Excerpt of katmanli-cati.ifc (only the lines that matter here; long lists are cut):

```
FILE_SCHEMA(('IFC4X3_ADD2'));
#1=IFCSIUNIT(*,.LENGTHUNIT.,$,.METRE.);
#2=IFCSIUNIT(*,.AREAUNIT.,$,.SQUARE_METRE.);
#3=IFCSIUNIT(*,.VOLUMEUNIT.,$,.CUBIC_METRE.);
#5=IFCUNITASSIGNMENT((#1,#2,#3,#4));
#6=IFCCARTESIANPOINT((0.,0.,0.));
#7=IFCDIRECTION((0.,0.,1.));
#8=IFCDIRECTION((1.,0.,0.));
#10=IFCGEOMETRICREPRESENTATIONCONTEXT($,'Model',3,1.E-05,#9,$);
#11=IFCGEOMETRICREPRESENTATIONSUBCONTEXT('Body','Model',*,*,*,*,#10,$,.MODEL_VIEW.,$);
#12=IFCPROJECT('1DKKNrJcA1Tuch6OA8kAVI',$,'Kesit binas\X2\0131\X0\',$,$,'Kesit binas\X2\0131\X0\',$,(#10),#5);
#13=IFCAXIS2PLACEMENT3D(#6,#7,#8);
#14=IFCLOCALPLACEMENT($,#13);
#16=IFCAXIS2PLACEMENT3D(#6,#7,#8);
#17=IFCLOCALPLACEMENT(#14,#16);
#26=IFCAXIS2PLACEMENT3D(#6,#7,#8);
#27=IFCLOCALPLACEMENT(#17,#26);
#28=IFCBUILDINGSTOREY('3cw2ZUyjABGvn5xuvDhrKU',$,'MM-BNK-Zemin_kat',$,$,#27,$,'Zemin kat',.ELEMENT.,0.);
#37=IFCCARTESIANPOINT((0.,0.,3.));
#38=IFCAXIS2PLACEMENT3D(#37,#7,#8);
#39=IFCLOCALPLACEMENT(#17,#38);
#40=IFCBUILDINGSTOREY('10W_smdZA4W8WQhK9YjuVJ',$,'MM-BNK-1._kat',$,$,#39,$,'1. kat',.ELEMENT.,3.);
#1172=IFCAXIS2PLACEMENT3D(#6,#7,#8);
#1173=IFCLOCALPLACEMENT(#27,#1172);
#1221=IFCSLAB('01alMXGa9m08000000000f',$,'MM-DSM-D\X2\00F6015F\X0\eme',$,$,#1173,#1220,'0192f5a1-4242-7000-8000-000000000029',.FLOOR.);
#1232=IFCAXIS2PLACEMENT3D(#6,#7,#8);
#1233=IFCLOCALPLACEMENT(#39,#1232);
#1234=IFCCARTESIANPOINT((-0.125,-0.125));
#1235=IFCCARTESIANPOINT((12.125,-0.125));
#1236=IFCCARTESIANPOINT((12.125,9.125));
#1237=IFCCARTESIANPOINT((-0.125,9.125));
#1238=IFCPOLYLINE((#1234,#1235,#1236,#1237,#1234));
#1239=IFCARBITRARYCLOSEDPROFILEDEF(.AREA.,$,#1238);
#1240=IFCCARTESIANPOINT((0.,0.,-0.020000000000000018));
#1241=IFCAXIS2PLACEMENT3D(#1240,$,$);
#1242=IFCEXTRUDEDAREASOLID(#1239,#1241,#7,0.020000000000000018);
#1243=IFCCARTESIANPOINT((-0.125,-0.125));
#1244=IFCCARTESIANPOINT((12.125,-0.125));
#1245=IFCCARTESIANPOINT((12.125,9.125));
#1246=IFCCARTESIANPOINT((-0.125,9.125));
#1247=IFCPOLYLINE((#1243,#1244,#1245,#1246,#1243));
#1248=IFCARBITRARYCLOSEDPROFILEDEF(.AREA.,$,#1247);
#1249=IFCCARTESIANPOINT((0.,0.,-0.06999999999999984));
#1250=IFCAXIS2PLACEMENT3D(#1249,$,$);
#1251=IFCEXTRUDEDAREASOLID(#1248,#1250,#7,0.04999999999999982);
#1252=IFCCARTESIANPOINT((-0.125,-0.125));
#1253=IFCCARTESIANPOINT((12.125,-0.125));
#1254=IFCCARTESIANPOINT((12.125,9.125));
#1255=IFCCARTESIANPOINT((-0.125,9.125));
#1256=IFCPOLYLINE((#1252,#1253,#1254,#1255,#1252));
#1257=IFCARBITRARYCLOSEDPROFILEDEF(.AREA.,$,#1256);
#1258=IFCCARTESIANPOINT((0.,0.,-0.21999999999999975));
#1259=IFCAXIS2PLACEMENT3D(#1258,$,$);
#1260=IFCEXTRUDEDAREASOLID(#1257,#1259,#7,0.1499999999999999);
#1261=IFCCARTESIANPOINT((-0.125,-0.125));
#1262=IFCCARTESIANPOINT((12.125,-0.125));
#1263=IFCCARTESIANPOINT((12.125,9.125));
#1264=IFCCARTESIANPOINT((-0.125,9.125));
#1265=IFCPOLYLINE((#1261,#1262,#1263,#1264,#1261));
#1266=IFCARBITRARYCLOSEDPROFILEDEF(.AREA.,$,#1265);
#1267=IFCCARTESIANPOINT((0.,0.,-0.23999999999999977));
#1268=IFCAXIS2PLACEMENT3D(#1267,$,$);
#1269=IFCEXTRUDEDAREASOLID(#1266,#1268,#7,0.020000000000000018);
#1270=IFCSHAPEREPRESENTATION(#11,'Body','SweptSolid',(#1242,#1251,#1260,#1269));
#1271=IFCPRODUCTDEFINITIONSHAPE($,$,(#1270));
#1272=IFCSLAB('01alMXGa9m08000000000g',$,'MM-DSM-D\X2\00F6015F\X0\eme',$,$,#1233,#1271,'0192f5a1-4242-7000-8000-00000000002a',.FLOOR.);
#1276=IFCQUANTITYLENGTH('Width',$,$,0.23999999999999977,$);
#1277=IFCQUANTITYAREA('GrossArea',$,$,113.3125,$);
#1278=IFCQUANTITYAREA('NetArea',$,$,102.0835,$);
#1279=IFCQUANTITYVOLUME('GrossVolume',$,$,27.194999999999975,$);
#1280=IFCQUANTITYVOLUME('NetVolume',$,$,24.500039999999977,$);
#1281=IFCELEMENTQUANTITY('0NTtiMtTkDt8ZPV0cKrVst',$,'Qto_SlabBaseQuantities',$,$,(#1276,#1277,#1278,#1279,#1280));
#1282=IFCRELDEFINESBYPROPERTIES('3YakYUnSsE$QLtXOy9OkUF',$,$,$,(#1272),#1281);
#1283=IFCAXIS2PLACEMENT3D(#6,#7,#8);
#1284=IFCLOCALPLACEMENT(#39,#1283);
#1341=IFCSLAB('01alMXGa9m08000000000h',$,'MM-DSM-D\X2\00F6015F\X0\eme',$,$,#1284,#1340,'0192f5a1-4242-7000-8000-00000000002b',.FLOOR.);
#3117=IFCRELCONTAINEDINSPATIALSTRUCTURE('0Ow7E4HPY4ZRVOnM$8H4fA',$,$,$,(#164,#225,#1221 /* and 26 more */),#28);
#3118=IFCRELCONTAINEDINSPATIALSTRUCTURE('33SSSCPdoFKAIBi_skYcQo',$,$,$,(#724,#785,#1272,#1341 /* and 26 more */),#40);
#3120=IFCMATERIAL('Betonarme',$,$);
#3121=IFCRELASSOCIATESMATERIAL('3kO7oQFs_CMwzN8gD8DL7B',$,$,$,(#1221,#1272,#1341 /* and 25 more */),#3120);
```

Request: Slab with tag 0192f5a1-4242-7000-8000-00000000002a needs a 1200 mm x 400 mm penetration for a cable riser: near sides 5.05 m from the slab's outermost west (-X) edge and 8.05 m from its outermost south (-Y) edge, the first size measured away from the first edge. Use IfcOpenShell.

```python
import numpy as np
import ifcopenshell
import ifcopenshell.api.feature
import ifcopenshell.api.geometry
import ifcopenshell.api.pset
import ifcopenshell.api.root
import ifcopenshell.geom
import ifcopenshell.util.element
import ifcopenshell.util.placement
import ifcopenshell.util.representation
import ifcopenshell.util.shape
import ifcopenshell.util.unit

model = ifcopenshell.open("katmanli-cati.ifc")
unit_scale = ifcopenshell.util.unit.calculate_unit_scale(model)
area_scale = ifcopenshell.util.unit.calculate_unit_scale(model, "AREAUNIT")
volume_scale = ifcopenshell.util.unit.calculate_unit_scale(model, "VOLUMEUNIT")
settings = ifcopenshell.geom.settings()


def volume(element):
    """Net volume in cubic metres, openings subtracted."""
    shape = ifcopenshell.geom.create_shape(settings, element)
    return ifcopenshell.util.shape.get_volume(shape.geometry)


slab = model.by_guid("01alMXGa9m08000000000g")
before = volume(slab)

# Extent in the slab's own axes, in metres. The edges named are its -X and -Y sides.
slab_shape = ifcopenshell.geom.create_shape(settings, slab)
vertices = ifcopenshell.util.shape.get_vertices(slab_shape.geometry)
x_min, y_min, bottom = vertices.min(axis=0)
top = vertices[:, 2].max()

opening = ifcopenshell.api.root.create_entity(model, ifc_class="IfcOpeningElement", name="Cable riser opening", predefined_type="OPENING")
context = ifcopenshell.util.representation.get_context(model, "Model", "Body", "MODEL_VIEW")
width, depth = 1.2, 0.4
outline = [(0.0, 0.0), (width, 0.0), (width, depth), (0.0, depth), (0.0, 0.0)]
# Overshoot both faces by 50 mm so the cut is clean.
shape = ifcopenshell.api.geometry.add_slab_representation(
    model, context=context, depth=top - bottom + 0.1, polyline=outline
)
ifcopenshell.api.geometry.assign_representation(model, product=opening, representation=shape)

matrix = ifcopenshell.util.placement.get_local_placement(slab.ObjectPlacement)
matrix[:, 3] = matrix @ np.append(np.array([x_min + 5.05, y_min + 8.05, bottom - 0.05]) / unit_scale, 1.0)
ifcopenshell.api.geometry.edit_object_placement(model, product=opening, matrix=matrix, is_si=False)
ifcopenshell.api.feature.add_feature(model, feature=opening, element=slab)

after = volume(slab)

# Update the slab's stored quantities.
qto = model.by_id(ifcopenshell.util.element.get_pset(slab, "Qto_SlabBaseQuantities", should_inherit=False)["id"])
ifcopenshell.api.pset.edit_qto(model, qto=qto, properties={
    "NetArea": after / (top - bottom) / area_scale,
    "NetVolume": after / volume_scale,
})

print(f"slab volume {before:.3f} -> {after:.3f} m3")

model.write("katmanli-cati_edited.ifc")
```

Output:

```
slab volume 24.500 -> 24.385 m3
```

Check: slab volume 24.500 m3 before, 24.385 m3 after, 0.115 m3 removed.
